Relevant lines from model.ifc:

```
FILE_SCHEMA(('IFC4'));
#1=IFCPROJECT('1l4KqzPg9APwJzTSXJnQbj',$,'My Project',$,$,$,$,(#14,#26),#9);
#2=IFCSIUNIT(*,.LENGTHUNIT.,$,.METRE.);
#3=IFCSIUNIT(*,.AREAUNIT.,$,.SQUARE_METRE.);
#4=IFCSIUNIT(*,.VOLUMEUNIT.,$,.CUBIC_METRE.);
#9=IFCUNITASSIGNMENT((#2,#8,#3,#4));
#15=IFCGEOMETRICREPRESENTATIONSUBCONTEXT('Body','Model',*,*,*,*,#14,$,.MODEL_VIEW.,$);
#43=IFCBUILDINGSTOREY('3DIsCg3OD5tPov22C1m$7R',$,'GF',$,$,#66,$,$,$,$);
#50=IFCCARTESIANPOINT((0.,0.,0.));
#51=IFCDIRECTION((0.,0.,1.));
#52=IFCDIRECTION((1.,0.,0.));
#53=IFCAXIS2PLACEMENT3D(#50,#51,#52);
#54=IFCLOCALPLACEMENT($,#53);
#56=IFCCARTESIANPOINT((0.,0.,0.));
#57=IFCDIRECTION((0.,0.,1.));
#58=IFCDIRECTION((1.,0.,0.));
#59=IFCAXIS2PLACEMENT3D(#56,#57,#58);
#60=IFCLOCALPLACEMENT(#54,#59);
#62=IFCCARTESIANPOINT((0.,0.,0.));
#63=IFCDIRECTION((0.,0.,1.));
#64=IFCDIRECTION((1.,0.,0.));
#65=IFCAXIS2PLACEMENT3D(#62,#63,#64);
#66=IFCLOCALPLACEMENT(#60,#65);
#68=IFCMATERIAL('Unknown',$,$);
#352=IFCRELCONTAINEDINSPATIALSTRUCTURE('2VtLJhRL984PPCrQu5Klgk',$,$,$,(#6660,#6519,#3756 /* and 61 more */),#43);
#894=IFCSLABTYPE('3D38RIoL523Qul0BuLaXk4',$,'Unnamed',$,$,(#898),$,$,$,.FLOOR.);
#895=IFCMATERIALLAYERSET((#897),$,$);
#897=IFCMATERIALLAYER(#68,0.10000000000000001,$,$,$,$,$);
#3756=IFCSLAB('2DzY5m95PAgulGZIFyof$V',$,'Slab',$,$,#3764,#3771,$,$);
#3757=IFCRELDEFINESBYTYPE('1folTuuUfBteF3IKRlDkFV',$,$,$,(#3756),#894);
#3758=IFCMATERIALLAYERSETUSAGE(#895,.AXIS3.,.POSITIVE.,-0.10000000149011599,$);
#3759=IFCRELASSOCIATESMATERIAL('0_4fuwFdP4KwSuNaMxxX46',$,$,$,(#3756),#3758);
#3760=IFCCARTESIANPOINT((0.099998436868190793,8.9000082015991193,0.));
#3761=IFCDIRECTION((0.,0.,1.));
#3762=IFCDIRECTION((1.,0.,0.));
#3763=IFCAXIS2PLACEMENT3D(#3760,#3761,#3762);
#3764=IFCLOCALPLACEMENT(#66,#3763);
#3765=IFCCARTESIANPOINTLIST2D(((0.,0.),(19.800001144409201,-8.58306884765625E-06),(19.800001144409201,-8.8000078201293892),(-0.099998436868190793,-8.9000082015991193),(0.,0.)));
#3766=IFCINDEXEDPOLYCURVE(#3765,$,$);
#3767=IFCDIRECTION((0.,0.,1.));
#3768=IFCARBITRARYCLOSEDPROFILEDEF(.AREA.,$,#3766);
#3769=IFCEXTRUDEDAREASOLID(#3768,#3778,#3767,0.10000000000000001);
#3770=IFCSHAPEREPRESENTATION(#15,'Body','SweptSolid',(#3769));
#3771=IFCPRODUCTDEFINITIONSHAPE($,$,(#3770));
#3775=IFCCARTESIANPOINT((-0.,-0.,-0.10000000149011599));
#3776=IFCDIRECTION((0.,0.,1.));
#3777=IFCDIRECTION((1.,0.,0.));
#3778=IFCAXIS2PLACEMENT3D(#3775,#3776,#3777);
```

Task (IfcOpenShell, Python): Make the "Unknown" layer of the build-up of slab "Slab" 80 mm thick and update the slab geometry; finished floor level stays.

```python
import ifcopenshell
import ifcopenshell.util.element
import ifcopenshell.util.representation

model = ifcopenshell.open("model.ifc")

layer_set = model.by_id(895)
layer = next(l for l in layer_set.MaterialLayers if l.Material and l.Material.Name == "Unknown")
change = 0.08 - layer.LayerThickness
layer.LayerThickness += change

# Geometry does not follow the layer set by itself.
slabs = [e for e in ifcopenshell.util.element.get_elements_by_material(model, layer_set) if e.is_a("IfcSlab")]
for slab in sorted(slabs, key=lambda e: e.id()):
    body = ifcopenshell.util.representation.get_representation(slab, "Model", "Body")
    solid = body.Items[0]
    old_depth = solid.Depth
    solid.Depth += change
    # Extruded upwards: lower the start of the extrusion so the top stays.
    x, y, z = solid.Position.Location.Coordinates
    solid.Position.Location = model.createIfcCartesianPoint((x, y, z - change))
    print(slab.id(), f"{old_depth:g} -> {solid.Depth:g}")

# The layers are counted up from the underside, which has moved.
for usage in {ifcopenshell.util.element.get_material(slab) for slab in slabs}:
    usage.OffsetFromReferenceLine -= change

model.write("model_rev.ifc")
```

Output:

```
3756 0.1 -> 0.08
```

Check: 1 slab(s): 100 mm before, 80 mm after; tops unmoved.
